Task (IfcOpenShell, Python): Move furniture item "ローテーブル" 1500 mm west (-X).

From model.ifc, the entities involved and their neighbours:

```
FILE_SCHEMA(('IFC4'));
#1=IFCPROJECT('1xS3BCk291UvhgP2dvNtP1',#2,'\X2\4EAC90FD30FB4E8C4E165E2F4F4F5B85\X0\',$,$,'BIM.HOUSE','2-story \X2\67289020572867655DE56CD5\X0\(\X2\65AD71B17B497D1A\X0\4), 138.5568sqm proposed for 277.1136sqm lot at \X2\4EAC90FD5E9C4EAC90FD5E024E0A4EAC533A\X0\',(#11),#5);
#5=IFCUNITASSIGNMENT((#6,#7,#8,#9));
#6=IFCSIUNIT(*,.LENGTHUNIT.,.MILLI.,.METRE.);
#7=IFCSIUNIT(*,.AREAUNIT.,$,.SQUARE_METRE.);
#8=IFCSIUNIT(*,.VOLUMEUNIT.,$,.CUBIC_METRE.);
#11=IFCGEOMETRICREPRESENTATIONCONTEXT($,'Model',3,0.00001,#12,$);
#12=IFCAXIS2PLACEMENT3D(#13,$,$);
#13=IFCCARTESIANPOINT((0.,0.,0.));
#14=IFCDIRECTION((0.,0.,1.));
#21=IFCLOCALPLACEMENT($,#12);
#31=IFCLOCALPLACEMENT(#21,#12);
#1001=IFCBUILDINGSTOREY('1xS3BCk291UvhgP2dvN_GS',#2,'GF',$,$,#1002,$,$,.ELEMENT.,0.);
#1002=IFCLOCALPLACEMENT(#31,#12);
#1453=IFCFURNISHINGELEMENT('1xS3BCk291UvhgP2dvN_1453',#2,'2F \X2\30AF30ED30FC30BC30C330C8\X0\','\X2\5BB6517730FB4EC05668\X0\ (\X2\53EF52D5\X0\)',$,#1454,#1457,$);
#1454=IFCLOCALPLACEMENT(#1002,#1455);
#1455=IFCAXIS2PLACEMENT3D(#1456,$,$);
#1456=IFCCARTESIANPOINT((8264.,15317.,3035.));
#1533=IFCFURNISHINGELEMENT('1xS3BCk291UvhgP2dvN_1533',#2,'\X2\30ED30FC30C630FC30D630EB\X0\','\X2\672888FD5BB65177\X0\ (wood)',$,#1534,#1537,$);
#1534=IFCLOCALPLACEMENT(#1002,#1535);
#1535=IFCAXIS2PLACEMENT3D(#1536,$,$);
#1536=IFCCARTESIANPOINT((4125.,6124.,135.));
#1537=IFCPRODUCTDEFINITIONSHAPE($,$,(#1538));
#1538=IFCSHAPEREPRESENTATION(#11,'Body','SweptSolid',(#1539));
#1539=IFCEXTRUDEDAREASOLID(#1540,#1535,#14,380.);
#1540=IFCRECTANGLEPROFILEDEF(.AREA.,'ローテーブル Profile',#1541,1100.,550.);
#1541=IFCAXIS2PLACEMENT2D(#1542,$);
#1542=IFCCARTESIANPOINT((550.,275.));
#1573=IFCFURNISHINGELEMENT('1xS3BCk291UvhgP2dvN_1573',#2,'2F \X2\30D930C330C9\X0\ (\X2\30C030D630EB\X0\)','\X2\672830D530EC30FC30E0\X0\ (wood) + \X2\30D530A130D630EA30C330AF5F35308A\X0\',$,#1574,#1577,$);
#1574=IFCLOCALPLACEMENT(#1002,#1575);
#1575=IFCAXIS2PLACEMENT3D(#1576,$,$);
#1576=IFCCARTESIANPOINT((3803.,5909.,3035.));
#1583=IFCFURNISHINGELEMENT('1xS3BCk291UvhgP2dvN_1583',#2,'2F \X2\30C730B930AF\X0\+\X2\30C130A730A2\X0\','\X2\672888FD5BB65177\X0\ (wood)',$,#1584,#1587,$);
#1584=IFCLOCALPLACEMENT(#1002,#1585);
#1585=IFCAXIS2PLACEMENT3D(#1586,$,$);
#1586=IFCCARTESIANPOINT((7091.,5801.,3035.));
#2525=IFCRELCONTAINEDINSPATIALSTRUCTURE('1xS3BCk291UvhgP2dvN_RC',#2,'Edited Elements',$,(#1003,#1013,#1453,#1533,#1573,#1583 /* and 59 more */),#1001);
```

```python
import ifcopenshell
import ifcopenshell.api.geometry
import ifcopenshell.util.placement
import ifcopenshell.util.unit

model = ifcopenshell.open("model.ifc")
unit_scale = ifcopenshell.util.unit.calculate_unit_scale(model)

item = model.by_id(1533)
matrix = ifcopenshell.util.placement.get_local_placement(item.ObjectPlacement)
matrix[0, 3] -= 1.5 / unit_scale
ifcopenshell.api.geometry.edit_object_placement(model, product=item, matrix=matrix, is_si=False)

print(ifcopenshell.util.placement.get_local_placement(item.ObjectPlacement).round(3) + 0.0)

model.write("model_edited.ifc")
```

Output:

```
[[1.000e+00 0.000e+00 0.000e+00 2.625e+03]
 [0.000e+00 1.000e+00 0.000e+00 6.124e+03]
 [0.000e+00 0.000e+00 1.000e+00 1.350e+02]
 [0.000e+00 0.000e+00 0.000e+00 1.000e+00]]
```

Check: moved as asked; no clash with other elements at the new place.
